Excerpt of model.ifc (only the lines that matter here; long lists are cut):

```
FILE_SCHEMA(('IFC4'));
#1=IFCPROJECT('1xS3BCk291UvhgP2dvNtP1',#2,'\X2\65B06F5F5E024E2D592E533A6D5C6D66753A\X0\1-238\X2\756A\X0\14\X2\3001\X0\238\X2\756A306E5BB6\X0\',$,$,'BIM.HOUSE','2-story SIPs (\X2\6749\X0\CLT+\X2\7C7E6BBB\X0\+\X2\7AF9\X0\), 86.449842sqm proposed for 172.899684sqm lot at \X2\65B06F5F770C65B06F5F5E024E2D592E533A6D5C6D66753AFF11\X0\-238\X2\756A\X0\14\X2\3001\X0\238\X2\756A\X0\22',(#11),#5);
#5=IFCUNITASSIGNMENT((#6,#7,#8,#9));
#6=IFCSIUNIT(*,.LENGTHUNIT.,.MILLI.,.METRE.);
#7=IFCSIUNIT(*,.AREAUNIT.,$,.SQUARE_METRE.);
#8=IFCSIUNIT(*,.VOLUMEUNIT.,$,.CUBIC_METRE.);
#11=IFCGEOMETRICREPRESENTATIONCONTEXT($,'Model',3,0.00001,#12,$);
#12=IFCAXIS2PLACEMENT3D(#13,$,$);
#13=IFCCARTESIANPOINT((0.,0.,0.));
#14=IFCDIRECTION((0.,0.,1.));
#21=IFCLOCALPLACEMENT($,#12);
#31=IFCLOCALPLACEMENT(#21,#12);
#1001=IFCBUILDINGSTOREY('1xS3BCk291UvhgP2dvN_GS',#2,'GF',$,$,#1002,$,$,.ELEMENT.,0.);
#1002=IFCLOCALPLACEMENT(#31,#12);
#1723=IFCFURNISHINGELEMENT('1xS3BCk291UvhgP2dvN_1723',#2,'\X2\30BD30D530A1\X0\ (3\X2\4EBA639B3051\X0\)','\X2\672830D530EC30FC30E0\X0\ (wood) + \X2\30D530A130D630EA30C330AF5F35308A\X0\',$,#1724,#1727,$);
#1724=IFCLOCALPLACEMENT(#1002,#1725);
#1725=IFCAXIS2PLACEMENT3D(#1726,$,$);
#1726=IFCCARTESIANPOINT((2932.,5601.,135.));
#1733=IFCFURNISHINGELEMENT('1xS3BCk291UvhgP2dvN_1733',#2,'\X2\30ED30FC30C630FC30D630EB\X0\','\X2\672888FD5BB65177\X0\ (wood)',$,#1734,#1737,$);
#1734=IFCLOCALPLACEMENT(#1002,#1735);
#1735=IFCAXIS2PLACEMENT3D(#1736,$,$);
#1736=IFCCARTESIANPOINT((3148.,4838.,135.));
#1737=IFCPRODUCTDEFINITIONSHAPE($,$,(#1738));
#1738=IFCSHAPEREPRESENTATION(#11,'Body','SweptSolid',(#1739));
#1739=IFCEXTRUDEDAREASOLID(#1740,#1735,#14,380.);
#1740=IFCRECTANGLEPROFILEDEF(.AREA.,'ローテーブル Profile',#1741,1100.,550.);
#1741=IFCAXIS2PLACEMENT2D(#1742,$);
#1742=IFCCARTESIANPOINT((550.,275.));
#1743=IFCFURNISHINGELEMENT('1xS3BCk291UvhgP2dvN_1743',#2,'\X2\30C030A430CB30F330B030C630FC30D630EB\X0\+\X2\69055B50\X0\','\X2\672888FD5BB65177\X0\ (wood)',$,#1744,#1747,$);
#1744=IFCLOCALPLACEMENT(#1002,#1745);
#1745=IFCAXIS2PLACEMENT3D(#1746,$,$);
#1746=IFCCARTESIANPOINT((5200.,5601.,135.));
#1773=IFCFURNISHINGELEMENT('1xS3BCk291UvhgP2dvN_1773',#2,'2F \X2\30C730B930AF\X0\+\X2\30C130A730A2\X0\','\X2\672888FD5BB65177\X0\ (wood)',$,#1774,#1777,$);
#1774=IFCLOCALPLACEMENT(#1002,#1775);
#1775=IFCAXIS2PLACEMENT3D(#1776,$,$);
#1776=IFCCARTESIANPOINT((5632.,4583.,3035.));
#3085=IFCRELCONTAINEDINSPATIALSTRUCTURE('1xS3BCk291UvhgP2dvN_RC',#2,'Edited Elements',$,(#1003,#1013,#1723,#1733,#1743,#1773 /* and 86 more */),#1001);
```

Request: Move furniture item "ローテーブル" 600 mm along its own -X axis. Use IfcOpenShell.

```python
import ifcopenshell
import ifcopenshell.api.geometry
import ifcopenshell.util.placement
import ifcopenshell.util.unit

model = ifcopenshell.open("model.ifc")
unit_scale = ifcopenshell.util.unit.calculate_unit_scale(model)

item = model.by_guid("1xS3BCk291UvhgP2dvN_1733")
matrix = ifcopenshell.util.placement.get_local_placement(item.ObjectPlacement)
matrix[:3, 3] -= matrix[:3, 0] * 0.6 / unit_scale
ifcopenshell.api.geometry.edit_object_placement(model, product=item, matrix=matrix, is_si=False)

print(ifcopenshell.util.placement.get_local_placement(item.ObjectPlacement).round(3) + 0.0)

model.write("model_v2.ifc")
```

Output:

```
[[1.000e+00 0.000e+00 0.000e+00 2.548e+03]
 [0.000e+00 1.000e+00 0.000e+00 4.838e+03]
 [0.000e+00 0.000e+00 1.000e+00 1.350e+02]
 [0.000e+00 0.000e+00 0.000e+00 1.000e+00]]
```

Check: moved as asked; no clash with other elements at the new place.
